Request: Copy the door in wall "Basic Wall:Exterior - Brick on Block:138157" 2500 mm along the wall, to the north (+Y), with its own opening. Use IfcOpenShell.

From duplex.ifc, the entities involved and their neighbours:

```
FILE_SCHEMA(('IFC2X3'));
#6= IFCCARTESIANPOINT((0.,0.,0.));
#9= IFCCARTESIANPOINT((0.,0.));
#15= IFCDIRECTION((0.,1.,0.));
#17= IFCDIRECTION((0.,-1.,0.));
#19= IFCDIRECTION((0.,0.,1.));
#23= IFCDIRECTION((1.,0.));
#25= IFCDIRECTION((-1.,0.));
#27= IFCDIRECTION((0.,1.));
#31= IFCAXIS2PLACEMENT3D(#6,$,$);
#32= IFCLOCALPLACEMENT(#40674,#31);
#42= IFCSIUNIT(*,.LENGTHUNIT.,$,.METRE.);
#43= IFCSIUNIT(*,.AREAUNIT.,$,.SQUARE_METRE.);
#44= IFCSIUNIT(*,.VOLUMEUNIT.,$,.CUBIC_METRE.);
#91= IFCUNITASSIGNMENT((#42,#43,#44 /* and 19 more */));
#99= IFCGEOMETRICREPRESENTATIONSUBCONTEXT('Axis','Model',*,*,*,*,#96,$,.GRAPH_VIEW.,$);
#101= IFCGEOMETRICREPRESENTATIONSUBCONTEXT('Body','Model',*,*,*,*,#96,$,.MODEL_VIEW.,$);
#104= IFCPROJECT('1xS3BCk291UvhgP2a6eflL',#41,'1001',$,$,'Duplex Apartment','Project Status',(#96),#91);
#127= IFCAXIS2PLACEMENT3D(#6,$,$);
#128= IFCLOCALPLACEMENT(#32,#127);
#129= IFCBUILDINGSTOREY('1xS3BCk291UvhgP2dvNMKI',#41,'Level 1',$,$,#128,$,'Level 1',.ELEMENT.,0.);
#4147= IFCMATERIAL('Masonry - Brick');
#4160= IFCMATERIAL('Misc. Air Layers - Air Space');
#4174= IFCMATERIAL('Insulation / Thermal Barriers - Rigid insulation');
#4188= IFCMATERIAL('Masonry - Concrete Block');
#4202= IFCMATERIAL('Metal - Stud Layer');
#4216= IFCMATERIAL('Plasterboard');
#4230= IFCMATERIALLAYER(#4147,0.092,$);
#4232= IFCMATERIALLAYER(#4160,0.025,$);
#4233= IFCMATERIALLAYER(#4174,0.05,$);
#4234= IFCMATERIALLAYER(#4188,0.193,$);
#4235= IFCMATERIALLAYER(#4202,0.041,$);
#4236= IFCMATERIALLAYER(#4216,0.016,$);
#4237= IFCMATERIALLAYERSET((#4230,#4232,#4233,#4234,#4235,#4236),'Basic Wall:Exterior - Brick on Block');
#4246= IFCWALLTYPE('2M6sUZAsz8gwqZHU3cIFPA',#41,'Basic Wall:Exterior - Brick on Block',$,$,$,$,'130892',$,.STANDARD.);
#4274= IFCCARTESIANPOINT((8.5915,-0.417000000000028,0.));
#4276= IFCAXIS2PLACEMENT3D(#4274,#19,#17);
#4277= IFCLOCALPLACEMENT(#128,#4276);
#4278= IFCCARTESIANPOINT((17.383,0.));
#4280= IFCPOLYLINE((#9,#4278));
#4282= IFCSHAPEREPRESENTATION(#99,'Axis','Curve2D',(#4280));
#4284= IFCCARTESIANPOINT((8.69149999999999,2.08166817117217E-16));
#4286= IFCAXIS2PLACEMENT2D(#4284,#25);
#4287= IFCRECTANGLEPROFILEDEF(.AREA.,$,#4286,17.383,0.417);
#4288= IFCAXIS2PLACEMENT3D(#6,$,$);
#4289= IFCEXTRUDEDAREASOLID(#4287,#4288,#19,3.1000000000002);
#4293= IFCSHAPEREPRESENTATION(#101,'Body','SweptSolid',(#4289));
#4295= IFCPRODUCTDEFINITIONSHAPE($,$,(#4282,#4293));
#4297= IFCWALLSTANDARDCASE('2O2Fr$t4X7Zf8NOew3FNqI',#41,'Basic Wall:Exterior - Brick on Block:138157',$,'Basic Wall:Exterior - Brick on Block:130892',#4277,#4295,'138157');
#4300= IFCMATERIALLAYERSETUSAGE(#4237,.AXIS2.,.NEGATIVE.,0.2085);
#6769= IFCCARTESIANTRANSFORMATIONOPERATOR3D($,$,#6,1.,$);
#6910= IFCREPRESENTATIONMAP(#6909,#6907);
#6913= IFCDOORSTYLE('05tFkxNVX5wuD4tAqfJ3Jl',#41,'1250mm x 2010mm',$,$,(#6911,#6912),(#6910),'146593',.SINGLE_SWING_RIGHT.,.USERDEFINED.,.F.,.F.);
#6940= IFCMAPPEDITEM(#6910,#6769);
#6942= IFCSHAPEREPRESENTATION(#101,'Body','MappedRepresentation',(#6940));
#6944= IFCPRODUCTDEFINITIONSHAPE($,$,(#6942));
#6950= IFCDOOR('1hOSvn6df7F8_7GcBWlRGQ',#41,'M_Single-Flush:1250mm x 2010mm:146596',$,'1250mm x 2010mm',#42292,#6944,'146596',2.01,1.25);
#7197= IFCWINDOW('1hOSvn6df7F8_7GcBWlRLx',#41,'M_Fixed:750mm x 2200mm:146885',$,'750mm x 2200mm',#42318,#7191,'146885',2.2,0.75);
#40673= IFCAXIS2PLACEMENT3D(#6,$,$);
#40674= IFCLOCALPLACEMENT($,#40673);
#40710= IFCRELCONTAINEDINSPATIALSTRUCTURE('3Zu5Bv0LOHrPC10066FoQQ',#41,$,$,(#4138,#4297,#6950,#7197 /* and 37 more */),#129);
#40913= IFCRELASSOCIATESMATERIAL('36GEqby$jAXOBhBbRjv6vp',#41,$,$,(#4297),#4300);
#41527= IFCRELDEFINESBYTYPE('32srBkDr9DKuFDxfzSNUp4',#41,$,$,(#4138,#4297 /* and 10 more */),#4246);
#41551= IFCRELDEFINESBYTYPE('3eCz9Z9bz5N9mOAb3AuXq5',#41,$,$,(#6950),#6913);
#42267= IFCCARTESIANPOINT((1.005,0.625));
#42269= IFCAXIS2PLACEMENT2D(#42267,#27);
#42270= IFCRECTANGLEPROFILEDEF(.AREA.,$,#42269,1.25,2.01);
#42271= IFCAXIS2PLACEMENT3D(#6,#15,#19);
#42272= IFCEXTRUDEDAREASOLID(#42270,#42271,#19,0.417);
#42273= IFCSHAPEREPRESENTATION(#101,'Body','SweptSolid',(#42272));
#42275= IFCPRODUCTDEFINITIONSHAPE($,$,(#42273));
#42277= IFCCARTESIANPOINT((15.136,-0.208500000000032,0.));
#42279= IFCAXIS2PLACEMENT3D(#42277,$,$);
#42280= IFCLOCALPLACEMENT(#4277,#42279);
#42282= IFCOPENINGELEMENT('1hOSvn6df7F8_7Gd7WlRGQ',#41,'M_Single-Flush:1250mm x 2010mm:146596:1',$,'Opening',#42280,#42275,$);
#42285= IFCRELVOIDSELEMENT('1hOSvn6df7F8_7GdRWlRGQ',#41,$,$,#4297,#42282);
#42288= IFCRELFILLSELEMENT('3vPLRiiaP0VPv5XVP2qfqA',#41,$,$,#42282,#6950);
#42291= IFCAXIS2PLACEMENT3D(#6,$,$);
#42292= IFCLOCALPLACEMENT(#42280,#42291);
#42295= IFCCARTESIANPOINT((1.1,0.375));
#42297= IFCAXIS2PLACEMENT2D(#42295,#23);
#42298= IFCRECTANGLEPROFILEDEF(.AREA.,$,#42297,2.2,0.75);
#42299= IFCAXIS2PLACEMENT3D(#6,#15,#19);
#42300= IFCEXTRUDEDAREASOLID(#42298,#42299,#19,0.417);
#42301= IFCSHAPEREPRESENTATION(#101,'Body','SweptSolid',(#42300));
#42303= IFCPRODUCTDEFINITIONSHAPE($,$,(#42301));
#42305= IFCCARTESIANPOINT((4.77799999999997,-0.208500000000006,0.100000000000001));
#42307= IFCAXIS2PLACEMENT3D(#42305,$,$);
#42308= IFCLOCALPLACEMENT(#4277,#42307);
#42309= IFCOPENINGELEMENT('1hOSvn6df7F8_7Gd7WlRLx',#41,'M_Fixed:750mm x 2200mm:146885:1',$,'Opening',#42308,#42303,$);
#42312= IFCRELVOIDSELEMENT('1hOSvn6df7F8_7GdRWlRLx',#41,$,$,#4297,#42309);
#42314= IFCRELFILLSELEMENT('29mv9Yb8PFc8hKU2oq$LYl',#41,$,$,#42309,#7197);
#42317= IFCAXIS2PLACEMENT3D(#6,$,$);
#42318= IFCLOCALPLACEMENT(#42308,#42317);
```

```python
import ifcopenshell
import ifcopenshell.api.feature
import ifcopenshell.api.geometry
import ifcopenshell.api.root
import ifcopenshell.geom
import ifcopenshell.util.element
import ifcopenshell.util.placement
import ifcopenshell.util.shape
import ifcopenshell.util.unit

model = ifcopenshell.open("duplex.ifc")
unit_scale = ifcopenshell.util.unit.calculate_unit_scale(model)
settings = ifcopenshell.geom.settings()


def volume(element):
    """Net volume in cubic metres, openings subtracted."""
    shape = ifcopenshell.geom.create_shape(settings, element)
    return ifcopenshell.util.shape.get_volume(shape.geometry)


def reuse_history(source, copy):
    """copy_class also copies each property set's owner history, people and application; keep the originals."""
    for rel in copy.IsDefinedBy:
        if rel.is_a("IfcRelDefinesByProperties") and (history := rel.RelatingPropertyDefinition.OwnerHistory):
            rel.RelatingPropertyDefinition.OwnerHistory = source.OwnerHistory
            ifcopenshell.util.element.remove_deep2(model, history)


door = model.by_guid("1hOSvn6df7F8_7GcBWlRGQ")
opening = door.FillsVoids[0].RelatingOpeningElement
wall = opening.VoidsElements[0].RelatingBuildingElement
before = volume(wall)
shift = ifcopenshell.util.placement.get_local_placement(wall.ObjectPlacement)[:3, 0] * -2.5 / unit_scale

# copy_class copies the void relationship, type, container and properties, but no geometry.
new_opening = ifcopenshell.api.root.copy_class(model, product=opening)
new_opening.Representation = ifcopenshell.util.element.copy_deep(
    model, opening.Representation, exclude=["IfcGeometricRepresentationContext", "IfcRepresentationMap"]
)
new_opening.Name = "M_Single-Flush:1250mm x 2010mm"
new_door = ifcopenshell.api.root.copy_class(model, product=door)
new_door.Representation = ifcopenshell.util.element.copy_deep(
    model, door.Representation, exclude=["IfcGeometricRepresentationContext", "IfcRepresentationMap"]
)
new_door.Name = "M_Single-Flush:1250mm x 2010mm"
new_door.Tag = None
reuse_history(door, new_door)
fills = ifcopenshell.api.feature.add_filling(model, opening=new_opening, element=new_door)
fills.OwnerHistory = new_door.OwnerHistory  # required in IFC2X3

for old, new in ((opening, new_opening), (door, new_door)):
    matrix = ifcopenshell.util.placement.get_local_placement(old.ObjectPlacement)
    matrix[:3, 3] += shift
    ifcopenshell.api.geometry.edit_object_placement(model, product=new, matrix=matrix, is_si=False)

after = volume(wall)

print(f"wall volume {before:.3f} -> {after:.3f} m3")

model.write("duplex_v2.ifc")
```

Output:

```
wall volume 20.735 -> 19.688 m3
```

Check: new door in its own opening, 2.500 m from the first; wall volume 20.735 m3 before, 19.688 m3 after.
